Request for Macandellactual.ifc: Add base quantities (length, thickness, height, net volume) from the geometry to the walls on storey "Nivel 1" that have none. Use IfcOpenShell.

First a look at what the model holds.

```python
import ifcopenshell
import ifcopenshell.util.element
import ifcopenshell.util.unit

model = ifcopenshell.open("Macandellactual.ifc")
print(model.schema)
for unit_type in ("LENGTHUNIT", "AREAUNIT", "VOLUMEUNIT"):
    print(unit_type, ifcopenshell.util.unit.calculate_unit_scale(model, unit_type))
storey = next(s for s in model.by_type("IfcBuildingStorey") if s.Name == "Nivel 1")
walls = [e for e in ifcopenshell.util.element.get_decomposition(storey) if e.is_a("IfcWall")]
for e in sorted(walls, key=lambda e: e.id()):
    print(e.id(), e.is_a(), e.Name, list(ifcopenshell.util.element.get_psets(e, qtos_only=True)), sep=" | ")
```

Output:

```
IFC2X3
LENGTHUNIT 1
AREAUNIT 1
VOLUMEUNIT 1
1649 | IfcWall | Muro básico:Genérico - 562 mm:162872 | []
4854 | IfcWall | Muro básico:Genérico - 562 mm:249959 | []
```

```python
import ifcopenshell
import ifcopenshell.api.pset
import ifcopenshell.geom
import ifcopenshell.util.element
import ifcopenshell.util.shape
import ifcopenshell.util.unit

model = ifcopenshell.open("Macandellactual.ifc")
unit_scale = ifcopenshell.util.unit.calculate_unit_scale(model)
volume_scale = ifcopenshell.util.unit.calculate_unit_scale(model, "VOLUMEUNIT")
settings = ifcopenshell.geom.settings()

storey = next(s for s in model.by_type("IfcBuildingStorey") if s.Name == "Nivel 1")
walls = [e for e in ifcopenshell.util.element.get_decomposition(storey) if e.is_a("IfcWall")]

for e in sorted(walls, key=lambda e: e.id()):
    if ifcopenshell.util.element.get_psets(e, qtos_only=True, should_inherit=False):
        continue
    # Geometry comes back in metres, in the element's own axes.
    shape = ifcopenshell.geom.create_shape(settings, e)
    values = {
        "Length": ifcopenshell.util.shape.get_x(shape.geometry) / unit_scale,
        "Width": ifcopenshell.util.shape.get_y(shape.geometry) / unit_scale,
        "Height": ifcopenshell.util.shape.get_z(shape.geometry) / unit_scale,
        "NetVolume": ifcopenshell.util.shape.get_volume(shape.geometry) / volume_scale,
    }
    qto = ifcopenshell.api.pset.add_qto(model, product=e, name="BaseQuantities")
    ifcopenshell.api.pset.edit_qto(model, qto=qto, properties=values)
    print(e.id(), {k: round(v, 3) for k, v in values.items()})

model.write("Macandellactual_edited.ifc")
```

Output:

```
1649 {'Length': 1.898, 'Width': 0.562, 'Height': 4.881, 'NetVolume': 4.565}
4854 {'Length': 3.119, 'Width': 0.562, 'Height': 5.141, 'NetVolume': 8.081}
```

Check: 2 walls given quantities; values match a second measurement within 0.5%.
